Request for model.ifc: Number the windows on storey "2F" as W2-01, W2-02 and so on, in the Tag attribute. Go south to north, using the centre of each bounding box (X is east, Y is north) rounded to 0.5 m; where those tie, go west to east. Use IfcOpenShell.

First a look at what the model holds.

```python
import ifcopenshell
import ifcopenshell.util.element
import ifcopenshell.util.placement

model = ifcopenshell.open("model.ifc")
print(model.schema)
storey = next(s for s in model.by_type("IfcBuildingStorey") if s.Name == "2F")
windows = [e for e in ifcopenshell.util.element.get_decomposition(storey) if e.is_a("IfcWindow")]
for e in sorted(windows, key=lambda e: e.id()):
    origin = ifcopenshell.util.placement.get_local_placement(e.ObjectPlacement)[:3, 3]
    print(e.id(), e.Tag, e.Name, origin.round(2) + 0.0, sep=" | ")
```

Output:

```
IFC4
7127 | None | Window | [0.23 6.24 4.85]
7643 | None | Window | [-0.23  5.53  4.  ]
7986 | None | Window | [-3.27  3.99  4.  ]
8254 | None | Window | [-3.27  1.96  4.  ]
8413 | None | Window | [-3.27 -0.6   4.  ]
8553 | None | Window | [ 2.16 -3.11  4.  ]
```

```python
import ifcopenshell
import ifcopenshell.geom
import ifcopenshell.util.element
import ifcopenshell.util.shape

model = ifcopenshell.open("model.ifc")
settings = ifcopenshell.geom.settings()
settings.set("use-world-coords", True)


def centre(element):
    shape = ifcopenshell.geom.create_shape(settings, element)
    return ifcopenshell.util.shape.get_bbox_centroid(shape.geometry)


storey = next(s for s in model.by_type("IfcBuildingStorey") if s.Name == "2F")
windows = [e for e in ifcopenshell.util.element.get_decomposition(storey) if e.is_a("IfcWindow")]

# Insertion points can sit at a corner or the storey origin, so sort by the geometry (in metres).
centres = {e: centre(e) for e in windows}
windows.sort(key=lambda e: (round(centres[e][1] / 0.5), centres[e][0]))

for i, e in enumerate(windows, start=1):
    number = f"W2-{i:02d}"
    e.Tag = number
    print(e.id(), number)

model.write("model_v2.ifc")
```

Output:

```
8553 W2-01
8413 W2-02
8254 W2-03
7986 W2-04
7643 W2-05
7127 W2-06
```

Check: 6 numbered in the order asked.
